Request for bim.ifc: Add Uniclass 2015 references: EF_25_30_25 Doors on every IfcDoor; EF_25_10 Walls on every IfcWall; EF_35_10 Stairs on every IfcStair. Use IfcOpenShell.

First a look at what the model holds.

```python
import ifcopenshell

model = ifcopenshell.open("bim.ifc")
print(model.schema)
print("classifications:", [c.Name for c in model.by_type("IfcClassification")])
for ifc_class in ("IfcDoor", "IfcRoof", "IfcStair", "IfcWall", "IfcWindow"):
    print(ifc_class, len(model.by_type(ifc_class)))
```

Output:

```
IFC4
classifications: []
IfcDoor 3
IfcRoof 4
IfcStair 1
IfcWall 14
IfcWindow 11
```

```python
import ifcopenshell
import ifcopenshell.api.classification

model = ifcopenshell.open("bim.ifc")

system = ifcopenshell.api.classification.add_classification(model, classification="Uniclass 2015")

codes = {
    "IfcDoor": ("EF_25_30_25", "Doors"),
    "IfcWall": ("EF_25_10", "Walls"),
    "IfcStair": ("EF_35_10", "Stairs"),
}
for ifc_class, (code, name) in codes.items():
    products = model.by_type(ifc_class)
    ifcopenshell.api.classification.add_reference(
        model, products=products, classification=system, identification=code, name=name
    )
    print(code, len(products))

model.write("bim_updated.ifc")
```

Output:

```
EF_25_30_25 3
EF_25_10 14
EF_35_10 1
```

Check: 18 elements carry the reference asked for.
